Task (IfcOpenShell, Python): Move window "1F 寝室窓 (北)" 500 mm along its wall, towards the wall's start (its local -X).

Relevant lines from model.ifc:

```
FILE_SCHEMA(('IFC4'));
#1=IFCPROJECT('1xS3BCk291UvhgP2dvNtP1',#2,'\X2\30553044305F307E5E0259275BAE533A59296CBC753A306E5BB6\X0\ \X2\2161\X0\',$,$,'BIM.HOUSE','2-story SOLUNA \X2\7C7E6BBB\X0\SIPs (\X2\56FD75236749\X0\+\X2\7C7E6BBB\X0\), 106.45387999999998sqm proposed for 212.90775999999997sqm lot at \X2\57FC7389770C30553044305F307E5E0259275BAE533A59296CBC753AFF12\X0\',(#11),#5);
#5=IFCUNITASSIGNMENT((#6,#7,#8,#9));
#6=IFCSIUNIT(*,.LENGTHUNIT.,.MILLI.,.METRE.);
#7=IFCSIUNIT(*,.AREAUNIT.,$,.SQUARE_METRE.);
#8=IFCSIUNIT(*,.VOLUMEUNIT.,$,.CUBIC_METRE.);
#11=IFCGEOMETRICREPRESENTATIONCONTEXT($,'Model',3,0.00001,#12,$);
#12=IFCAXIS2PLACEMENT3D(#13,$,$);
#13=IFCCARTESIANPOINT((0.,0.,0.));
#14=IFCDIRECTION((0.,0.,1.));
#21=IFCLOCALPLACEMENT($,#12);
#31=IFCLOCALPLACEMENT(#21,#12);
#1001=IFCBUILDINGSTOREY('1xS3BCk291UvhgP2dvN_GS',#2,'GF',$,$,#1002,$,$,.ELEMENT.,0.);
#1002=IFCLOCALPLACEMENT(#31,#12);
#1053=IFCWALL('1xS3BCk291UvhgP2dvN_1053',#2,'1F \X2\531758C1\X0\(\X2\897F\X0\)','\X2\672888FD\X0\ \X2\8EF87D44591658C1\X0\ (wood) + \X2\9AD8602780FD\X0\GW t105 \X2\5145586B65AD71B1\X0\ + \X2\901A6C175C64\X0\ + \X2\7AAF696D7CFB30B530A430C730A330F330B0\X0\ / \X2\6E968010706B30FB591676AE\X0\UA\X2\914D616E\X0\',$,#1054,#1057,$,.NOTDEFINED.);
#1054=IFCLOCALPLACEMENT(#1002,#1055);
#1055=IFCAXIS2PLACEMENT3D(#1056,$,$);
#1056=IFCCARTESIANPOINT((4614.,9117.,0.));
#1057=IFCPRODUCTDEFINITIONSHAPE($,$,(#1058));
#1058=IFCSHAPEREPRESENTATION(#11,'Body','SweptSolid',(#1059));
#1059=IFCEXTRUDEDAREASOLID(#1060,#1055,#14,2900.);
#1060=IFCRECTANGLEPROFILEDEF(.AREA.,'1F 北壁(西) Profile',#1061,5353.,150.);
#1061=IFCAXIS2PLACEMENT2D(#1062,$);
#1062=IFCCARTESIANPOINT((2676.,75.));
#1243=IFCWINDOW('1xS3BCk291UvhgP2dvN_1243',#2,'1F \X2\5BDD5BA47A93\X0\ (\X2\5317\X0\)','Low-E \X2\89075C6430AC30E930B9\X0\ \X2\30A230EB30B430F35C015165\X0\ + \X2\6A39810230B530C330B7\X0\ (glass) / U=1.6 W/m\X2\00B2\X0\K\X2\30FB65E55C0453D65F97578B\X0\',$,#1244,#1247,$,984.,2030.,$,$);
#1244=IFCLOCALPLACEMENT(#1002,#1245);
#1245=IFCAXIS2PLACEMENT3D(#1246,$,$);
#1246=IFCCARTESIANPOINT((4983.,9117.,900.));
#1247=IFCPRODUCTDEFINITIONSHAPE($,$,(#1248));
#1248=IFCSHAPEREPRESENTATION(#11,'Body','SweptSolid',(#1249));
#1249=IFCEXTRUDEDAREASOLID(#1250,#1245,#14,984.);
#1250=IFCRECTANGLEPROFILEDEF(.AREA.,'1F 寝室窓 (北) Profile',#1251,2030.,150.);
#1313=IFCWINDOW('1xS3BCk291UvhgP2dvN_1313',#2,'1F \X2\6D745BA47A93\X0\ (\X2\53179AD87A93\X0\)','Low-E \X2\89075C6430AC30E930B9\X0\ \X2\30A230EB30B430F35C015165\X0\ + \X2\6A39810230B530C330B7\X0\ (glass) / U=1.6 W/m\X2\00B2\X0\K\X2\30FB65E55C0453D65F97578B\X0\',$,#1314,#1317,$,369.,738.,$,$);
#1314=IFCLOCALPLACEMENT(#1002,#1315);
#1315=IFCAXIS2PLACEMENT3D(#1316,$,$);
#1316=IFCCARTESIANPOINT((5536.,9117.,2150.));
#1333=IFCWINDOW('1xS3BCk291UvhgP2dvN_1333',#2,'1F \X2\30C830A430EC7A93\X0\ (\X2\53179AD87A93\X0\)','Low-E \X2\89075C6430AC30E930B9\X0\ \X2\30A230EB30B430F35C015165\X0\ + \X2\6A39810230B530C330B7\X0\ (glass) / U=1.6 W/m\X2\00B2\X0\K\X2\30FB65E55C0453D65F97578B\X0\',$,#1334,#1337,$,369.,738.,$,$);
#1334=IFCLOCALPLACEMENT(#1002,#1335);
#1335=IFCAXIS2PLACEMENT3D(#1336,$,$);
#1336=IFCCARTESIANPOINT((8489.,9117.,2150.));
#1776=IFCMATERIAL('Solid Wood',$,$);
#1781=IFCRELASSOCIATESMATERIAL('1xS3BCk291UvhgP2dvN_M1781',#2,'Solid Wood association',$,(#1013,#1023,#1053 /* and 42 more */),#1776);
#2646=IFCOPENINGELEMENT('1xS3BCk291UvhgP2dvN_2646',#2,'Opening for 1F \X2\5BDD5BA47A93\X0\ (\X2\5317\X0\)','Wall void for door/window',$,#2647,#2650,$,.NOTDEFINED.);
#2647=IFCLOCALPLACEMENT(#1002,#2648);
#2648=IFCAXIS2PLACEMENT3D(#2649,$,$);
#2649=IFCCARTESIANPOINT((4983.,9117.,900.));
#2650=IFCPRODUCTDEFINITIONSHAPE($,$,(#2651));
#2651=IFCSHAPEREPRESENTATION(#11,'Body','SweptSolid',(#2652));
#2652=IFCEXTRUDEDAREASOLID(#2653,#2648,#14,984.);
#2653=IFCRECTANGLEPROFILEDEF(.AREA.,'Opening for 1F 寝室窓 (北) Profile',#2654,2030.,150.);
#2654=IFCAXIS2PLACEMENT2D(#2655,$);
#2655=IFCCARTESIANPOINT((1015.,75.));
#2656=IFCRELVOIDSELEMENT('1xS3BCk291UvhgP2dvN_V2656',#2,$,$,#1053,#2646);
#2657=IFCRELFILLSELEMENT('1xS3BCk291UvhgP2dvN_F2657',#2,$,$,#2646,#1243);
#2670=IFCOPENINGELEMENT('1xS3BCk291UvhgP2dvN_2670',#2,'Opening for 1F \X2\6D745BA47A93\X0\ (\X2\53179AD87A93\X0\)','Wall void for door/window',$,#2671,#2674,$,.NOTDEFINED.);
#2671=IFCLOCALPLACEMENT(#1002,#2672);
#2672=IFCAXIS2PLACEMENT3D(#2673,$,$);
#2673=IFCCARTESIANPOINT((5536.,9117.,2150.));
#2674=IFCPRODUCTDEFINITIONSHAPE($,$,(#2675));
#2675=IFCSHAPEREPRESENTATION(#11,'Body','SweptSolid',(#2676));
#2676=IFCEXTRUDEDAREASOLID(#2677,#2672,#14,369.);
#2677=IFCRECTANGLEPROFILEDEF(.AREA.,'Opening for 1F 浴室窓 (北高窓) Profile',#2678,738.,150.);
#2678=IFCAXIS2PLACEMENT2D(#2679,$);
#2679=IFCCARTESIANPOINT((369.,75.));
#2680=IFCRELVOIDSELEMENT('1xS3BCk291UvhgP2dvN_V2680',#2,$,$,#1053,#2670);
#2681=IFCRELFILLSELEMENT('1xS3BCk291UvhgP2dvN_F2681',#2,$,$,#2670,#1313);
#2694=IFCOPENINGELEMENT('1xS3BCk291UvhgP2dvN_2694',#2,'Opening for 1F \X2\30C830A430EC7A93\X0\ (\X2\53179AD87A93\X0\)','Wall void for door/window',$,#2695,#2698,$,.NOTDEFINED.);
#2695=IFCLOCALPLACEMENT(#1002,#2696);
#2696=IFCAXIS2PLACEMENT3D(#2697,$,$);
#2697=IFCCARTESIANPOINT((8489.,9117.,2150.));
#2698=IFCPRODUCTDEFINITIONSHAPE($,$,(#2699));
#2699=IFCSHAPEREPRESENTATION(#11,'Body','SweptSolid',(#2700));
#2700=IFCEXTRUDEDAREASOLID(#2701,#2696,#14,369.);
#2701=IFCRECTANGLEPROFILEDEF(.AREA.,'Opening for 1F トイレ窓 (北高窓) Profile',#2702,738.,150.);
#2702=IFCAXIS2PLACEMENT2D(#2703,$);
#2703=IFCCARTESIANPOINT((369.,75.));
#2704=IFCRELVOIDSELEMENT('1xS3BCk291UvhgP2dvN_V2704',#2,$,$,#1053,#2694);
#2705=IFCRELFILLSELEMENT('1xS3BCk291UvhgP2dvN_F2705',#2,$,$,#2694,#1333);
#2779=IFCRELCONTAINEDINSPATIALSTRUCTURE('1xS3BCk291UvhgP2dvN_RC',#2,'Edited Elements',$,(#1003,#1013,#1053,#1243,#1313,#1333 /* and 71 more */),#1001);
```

```python
import ifcopenshell
import ifcopenshell.api.geometry
import ifcopenshell.util.placement
import ifcopenshell.util.unit

model = ifcopenshell.open("model.ifc")
unit_scale = ifcopenshell.util.unit.calculate_unit_scale(model)

window = model.by_id(1243)
opening = window.FillsVoids[0].RelatingOpeningElement
wall = opening.VoidsElements[0].RelatingBuildingElement

wall_matrix = ifcopenshell.util.placement.get_local_placement(wall.ObjectPlacement)
shift = wall_matrix[:3, 0] * -0.5 / unit_scale
before = ifcopenshell.util.placement.get_local_placement(window.ObjectPlacement)[:3, 3].copy()

# The window is not placed relative to its opening, so move both.
for product in (opening, window):
    matrix = ifcopenshell.util.placement.get_local_placement(product.ObjectPlacement)
    matrix[:3, 3] += shift
    ifcopenshell.api.geometry.edit_object_placement(model, product=product, matrix=matrix, is_si=False)

after = ifcopenshell.util.placement.get_local_placement(window.ObjectPlacement)[:3, 3]
print("window moved by", (after - before).round(3) + 0.0)

model.write("model-out.ifc")
```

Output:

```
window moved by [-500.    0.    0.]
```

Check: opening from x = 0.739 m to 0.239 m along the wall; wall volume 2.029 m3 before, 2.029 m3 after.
